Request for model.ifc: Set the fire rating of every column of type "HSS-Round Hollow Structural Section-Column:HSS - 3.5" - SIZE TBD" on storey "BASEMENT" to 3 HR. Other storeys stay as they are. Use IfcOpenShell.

First a look at what the model holds.

```python
import ifcopenshell
import ifcopenshell.util.element

model = ifcopenshell.open("model.ifc")
print(model.schema)
storey = next(s for s in model.by_type("IfcBuildingStorey") if s.Name == "BASEMENT")
columns = [e for e in ifcopenshell.util.element.get_decomposition(storey) if e.is_a("IfcColumn")]
seen = {}
for e in columns:
    element_type = ifcopenshell.util.element.get_type(e)
    key = (element_type.Name if element_type != e and element_type else None, ifcopenshell.util.element.get_pset(e, "Pset_ColumnCommon", "FireRating"))
    seen[key] = seen.get(key, 0) + 1
for (name, value), count in sorted(seen.items(), key=str):
    print(count, "x", name, "|", value)
```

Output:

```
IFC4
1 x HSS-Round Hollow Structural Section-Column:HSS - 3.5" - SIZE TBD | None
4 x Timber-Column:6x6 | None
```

```python
import ifcopenshell
import ifcopenshell.api.pset
import ifcopenshell.util.element

model = ifcopenshell.open("model.ifc")

storey = next(s for s in model.by_type("IfcBuildingStorey") if s.Name == "BASEMENT")
columns = [e for e in ifcopenshell.util.element.get_decomposition(storey) if e.is_a("IfcColumn")]

count = 0
for e in columns:
    element_type = ifcopenshell.util.element.get_type(e)
    if element_type in (None, e) or element_type.Name != 'HSS-Round Hollow Structural Section-Column:HSS - 3.5" - SIZE TBD':
        continue
    # add_pset returns the element's existing set when there is one.
    pset = ifcopenshell.api.pset.add_pset(model, product=e, name="Pset_ColumnCommon")
    ifcopenshell.api.pset.edit_pset(model, pset=pset, properties={"FireRating": "3 HR"})
    count += 1

print(count, "columns updated")

model.write("model_v2.ifc")
```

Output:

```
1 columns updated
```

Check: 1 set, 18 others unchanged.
